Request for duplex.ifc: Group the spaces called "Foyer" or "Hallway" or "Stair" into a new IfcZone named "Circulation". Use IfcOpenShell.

First a look at what the model holds.

```python
import ifcopenshell

model = ifcopenshell.open("duplex.ifc")
print(model.schema)
seen = {}
for space in model.by_type("IfcSpace"):
    seen[space.LongName] = seen.get(space.LongName, 0) + 1
for name, count in sorted(seen.items(), key=str):
    print(count, "x", name)
print("zones:", [z.Name for z in model.by_type("IfcZone")][:20])
```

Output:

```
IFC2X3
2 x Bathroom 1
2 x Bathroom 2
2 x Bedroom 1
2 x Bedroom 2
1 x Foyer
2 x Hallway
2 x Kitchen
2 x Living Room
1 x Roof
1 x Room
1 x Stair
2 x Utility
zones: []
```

```python
import ifcopenshell
import ifcopenshell.api.group
import ifcopenshell.api.root

model = ifcopenshell.open("duplex.ifc")

names = {"Foyer", "Hallway", "Stair"}
spaces = [s for s in model.by_type("IfcSpace") if s.LongName in names]

zone = ifcopenshell.api.root.create_entity(model, ifc_class="IfcZone", name="Circulation")
ifcopenshell.api.group.assign_group(model, products=spaces, group=zone)
print(len(spaces), "spaces in", zone.Name)

model.write("duplex_updated.ifc")
```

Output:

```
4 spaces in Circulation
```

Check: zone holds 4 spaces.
